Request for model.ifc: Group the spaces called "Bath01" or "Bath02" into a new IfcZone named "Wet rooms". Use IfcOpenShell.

First a look at what the model holds.

```python
import ifcopenshell

model = ifcopenshell.open("model.ifc")
print(model.schema)
seen = {}
for space in model.by_type("IfcSpace"):
    seen[space.Name] = seen.get(space.Name, 0) + 1
for name, count in sorted(seen.items(), key=str):
    print(count, "x", name)
print("zones:", [z.Name for z in model.by_type("IfcZone")][:20])
```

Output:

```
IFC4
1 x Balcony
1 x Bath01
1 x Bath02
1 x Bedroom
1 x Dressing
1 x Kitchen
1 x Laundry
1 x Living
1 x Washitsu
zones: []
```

```python
import ifcopenshell
import ifcopenshell.api.group
import ifcopenshell.api.root

model = ifcopenshell.open("model.ifc")

names = {"Bath01", "Bath02"}
spaces = [s for s in model.by_type("IfcSpace") if s.Name in names]

zone = ifcopenshell.api.root.create_entity(model, ifc_class="IfcZone", name="Wet rooms")
ifcopenshell.api.group.assign_group(model, products=spaces, group=zone)
print(len(spaces), "spaces in", zone.Name)

model.write("model_rev.ifc")
```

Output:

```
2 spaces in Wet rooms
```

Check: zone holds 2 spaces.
